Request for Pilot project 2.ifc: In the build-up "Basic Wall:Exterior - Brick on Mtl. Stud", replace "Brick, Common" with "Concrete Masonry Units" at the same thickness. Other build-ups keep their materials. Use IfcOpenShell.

First a look at what the model holds.

```python
import ifcopenshell
import ifcopenshell.util.element

model = ifcopenshell.open("Pilot project 2.ifc")
print(model.schema)
for layer_set in model.by_type("IfcMaterialLayerSet"):
    if layer_set.LayerSetName == "Basic Wall:Exterior - Brick on Mtl. Stud":
        for layer in layer_set.MaterialLayers:
            print(layer.id(), layer.Material and layer.Material.Name, layer.LayerThickness, sep=" | ")
        print(len(ifcopenshell.util.element.get_elements_by_material(model, layer_set)), "elements and types use it")
print(sorted(m.Name for m in model.by_type("IfcMaterial") if m.Name)[:60])
```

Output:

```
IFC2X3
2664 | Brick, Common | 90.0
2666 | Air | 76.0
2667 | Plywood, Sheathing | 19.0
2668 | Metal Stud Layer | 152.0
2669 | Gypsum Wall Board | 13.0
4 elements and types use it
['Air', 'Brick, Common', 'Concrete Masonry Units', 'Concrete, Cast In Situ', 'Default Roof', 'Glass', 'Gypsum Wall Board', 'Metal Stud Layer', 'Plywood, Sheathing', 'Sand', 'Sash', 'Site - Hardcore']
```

```python
import ifcopenshell
import ifcopenshell.api.material

model = ifcopenshell.open("Pilot project 2.ifc")

layer_set = next(s for s in model.by_type("IfcMaterialLayerSet") if s.LayerSetName == "Basic Wall:Exterior - Brick on Mtl. Stud")
layer = next(l for l in layer_set.MaterialLayers if l.Material and l.Material.Name == "Brick, Common")
material = next(m for m in model.by_type("IfcMaterial") if m.Name == "Concrete Masonry Units")

# Point this one layer at the other material; renaming the old one would change it everywhere.
ifcopenshell.api.material.edit_layer(model, layer=layer, attributes={}, material=material)

print([l.Material.Name if l.Material else None for l in layer_set.MaterialLayers])

model.write("Pilot project 2_edited.ifc")
```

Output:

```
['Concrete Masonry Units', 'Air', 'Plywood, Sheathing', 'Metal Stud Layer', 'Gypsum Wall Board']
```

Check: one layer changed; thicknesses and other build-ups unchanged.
